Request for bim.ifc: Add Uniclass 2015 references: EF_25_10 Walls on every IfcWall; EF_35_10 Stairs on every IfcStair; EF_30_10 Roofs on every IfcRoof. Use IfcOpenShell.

First a look at what the model holds.

```python
import ifcopenshell

model = ifcopenshell.open("bim.ifc")
print(model.schema)
print("classifications:", [c.Name for c in model.by_type("IfcClassification")])
for ifc_class in ("IfcDoor", "IfcRoof", "IfcStair", "IfcWall", "IfcWindow"):
    print(ifc_class, len(model.by_type(ifc_class)))
```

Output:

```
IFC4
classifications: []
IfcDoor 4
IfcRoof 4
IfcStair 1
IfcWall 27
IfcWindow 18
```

```python
import ifcopenshell
import ifcopenshell.api.classification

model = ifcopenshell.open("bim.ifc")

system = ifcopenshell.api.classification.add_classification(model, classification="Uniclass 2015")

codes = {
    "IfcWall": ("EF_25_10", "Walls"),
    "IfcStair": ("EF_35_10", "Stairs"),
    "IfcRoof": ("EF_30_10", "Roofs"),
}
for ifc_class, (code, name) in codes.items():
    products = model.by_type(ifc_class)
    ifcopenshell.api.classification.add_reference(
        model, products=products, classification=system, identification=code, name=name
    )
    print(code, len(products))

model.write("bim_v2.ifc")
```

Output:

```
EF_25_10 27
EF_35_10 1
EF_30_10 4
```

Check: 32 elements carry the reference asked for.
